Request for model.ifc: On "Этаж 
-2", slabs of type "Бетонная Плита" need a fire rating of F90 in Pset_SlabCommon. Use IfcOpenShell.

First a look at what the model holds.

```python
import ifcopenshell
import ifcopenshell.util.element

model = ifcopenshell.open("model.ifc")
print(model.schema)
storey = next(s for s in model.by_type("IfcBuildingStorey") if s.Name == 'Этаж \r\n-2')
slabs = [e for e in ifcopenshell.util.element.get_decomposition(storey) if e.is_a("IfcSlab")]
seen = {}
for e in slabs:
    element_type = ifcopenshell.util.element.get_type(e)
    key = (element_type.Name if element_type != e and element_type else None, ifcopenshell.util.element.get_pset(e, "Pset_SlabCommon", "FireRating"))
    seen[key] = seen.get(key, 0) + 1
for (name, value), count in sorted(seen.items(), key=str):
    print(count, "x", name, "|", value)
```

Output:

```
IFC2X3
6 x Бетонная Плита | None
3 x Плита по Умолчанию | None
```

```python
import ifcopenshell
import ifcopenshell.api.pset
import ifcopenshell.util.element

model = ifcopenshell.open("model.ifc")

storey = next(s for s in model.by_type("IfcBuildingStorey") if s.Name == 'Этаж \r\n-2')
slabs = [e for e in ifcopenshell.util.element.get_decomposition(storey) if e.is_a("IfcSlab")]

count = 0
for e in slabs:
    element_type = ifcopenshell.util.element.get_type(e)
    if element_type in (None, e) or element_type.Name != "Бетонная Плита":
        continue
    # add_pset returns the element's existing set when there is one.
    pset = ifcopenshell.api.pset.add_pset(model, product=e, name="Pset_SlabCommon")
    ifcopenshell.api.pset.edit_pset(model, pset=pset, properties={"FireRating": "F90"})
    count += 1

print(count, "slabs updated")

model.write("model_edited.ifc")
```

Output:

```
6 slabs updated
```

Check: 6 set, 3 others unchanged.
